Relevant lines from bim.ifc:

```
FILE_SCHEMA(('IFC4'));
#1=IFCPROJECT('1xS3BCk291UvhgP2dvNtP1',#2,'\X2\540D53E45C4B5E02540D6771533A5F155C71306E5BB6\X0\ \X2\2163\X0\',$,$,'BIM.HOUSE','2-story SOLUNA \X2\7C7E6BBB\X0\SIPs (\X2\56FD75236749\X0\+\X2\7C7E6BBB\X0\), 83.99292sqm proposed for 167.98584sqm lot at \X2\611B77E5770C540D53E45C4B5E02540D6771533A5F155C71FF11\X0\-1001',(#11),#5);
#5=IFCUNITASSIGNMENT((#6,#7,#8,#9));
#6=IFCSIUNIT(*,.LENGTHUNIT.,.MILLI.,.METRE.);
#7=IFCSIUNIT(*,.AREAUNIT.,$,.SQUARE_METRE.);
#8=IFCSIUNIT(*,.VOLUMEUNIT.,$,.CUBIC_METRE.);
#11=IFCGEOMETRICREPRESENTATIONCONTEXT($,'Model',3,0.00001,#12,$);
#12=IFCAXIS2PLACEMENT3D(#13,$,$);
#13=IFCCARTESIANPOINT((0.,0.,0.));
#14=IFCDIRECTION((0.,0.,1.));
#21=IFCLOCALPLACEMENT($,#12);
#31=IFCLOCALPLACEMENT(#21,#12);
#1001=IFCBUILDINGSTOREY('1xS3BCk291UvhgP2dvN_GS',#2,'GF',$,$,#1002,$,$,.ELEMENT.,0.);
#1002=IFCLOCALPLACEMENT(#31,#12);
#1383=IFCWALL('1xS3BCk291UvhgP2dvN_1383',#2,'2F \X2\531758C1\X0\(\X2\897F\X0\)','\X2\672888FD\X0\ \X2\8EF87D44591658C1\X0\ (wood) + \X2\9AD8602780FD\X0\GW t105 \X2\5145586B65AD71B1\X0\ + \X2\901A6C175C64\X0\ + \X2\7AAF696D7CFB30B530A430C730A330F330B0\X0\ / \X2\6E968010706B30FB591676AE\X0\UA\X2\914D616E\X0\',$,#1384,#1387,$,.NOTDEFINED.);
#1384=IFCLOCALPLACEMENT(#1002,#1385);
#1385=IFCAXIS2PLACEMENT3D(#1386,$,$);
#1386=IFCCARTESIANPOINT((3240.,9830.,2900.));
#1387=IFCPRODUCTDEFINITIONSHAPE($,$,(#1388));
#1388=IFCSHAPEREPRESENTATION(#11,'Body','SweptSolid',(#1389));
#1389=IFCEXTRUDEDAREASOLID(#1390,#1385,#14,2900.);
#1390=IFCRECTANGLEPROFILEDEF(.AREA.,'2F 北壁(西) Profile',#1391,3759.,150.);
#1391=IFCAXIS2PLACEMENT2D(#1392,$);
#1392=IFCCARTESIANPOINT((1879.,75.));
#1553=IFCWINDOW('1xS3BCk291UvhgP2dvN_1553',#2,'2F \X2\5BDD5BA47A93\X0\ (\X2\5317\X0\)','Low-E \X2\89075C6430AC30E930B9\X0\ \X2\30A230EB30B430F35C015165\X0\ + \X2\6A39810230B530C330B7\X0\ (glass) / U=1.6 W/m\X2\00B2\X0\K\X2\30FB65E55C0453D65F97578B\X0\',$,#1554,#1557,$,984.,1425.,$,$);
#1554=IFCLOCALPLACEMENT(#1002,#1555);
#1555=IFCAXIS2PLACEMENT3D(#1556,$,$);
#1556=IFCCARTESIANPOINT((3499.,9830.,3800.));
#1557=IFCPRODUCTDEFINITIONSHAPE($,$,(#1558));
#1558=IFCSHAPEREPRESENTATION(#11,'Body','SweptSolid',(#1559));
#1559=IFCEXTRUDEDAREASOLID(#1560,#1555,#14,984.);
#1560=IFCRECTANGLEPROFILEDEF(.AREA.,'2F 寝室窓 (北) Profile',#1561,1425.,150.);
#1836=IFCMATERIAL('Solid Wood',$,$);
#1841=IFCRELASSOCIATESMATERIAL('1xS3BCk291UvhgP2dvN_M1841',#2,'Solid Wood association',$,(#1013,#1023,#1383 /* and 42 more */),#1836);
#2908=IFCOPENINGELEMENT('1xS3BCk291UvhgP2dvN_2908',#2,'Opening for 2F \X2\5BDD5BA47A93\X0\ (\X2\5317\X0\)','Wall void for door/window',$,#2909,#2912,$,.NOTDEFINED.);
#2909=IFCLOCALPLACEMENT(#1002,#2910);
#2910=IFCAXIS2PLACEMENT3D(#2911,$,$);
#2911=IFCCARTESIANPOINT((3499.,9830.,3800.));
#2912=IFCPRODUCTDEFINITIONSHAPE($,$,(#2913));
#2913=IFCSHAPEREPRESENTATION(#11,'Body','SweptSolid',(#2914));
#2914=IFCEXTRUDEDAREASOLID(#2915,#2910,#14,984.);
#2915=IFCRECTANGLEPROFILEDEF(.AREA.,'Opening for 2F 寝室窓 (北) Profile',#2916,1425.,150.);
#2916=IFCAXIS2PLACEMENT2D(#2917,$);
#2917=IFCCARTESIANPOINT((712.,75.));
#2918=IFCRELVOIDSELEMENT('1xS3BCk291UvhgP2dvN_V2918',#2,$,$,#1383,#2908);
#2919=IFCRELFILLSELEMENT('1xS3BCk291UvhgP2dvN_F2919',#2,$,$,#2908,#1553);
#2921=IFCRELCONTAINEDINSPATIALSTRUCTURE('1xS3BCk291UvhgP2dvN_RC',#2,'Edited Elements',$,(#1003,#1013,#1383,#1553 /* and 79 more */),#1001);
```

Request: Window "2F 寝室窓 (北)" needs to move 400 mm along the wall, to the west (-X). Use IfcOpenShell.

```python
import ifcopenshell
import ifcopenshell.api.geometry
import ifcopenshell.util.placement
import ifcopenshell.util.unit

model = ifcopenshell.open("bim.ifc")
unit_scale = ifcopenshell.util.unit.calculate_unit_scale(model)

window = model.by_guid("1xS3BCk291UvhgP2dvN_1553")
opening = window.FillsVoids[0].RelatingOpeningElement
wall = opening.VoidsElements[0].RelatingBuildingElement

wall_matrix = ifcopenshell.util.placement.get_local_placement(wall.ObjectPlacement)
shift = wall_matrix[:3, 0] * -0.4 / unit_scale
before = ifcopenshell.util.placement.get_local_placement(window.ObjectPlacement)[:3, 3].copy()

# The window is not placed relative to its opening, so move both.
for product in (opening, window):
    matrix = ifcopenshell.util.placement.get_local_placement(product.ObjectPlacement)
    matrix[:3, 3] += shift
    ifcopenshell.api.geometry.edit_object_placement(model, product=product, matrix=matrix, is_si=False)

after = ifcopenshell.util.placement.get_local_placement(window.ObjectPlacement)[:3, 3]
print("window moved by", (after - before).round(3) + 0.0)

model.write("bim_rev.ifc")
```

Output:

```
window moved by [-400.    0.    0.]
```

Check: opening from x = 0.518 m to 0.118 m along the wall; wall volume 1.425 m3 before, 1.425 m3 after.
